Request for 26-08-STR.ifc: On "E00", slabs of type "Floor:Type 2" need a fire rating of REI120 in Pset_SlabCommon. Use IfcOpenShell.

First a look at what the model holds.

```python
import ifcopenshell
import ifcopenshell.util.element

model = ifcopenshell.open("26-08-STR.ifc")
print(model.schema)
storey = next(s for s in model.by_type("IfcBuildingStorey") if s.Name == "E00")
slabs = [e for e in ifcopenshell.util.element.get_decomposition(storey) if e.is_a("IfcSlab")]
seen = {}
for e in slabs:
    element_type = ifcopenshell.util.element.get_type(e)
    key = (element_type.Name if element_type != e and element_type else None, ifcopenshell.util.element.get_pset(e, "Pset_SlabCommon", "FireRating"))
    seen[key] = seen.get(key, 0) + 1
for (name, value), count in sorted(seen.items(), key=str):
    print(count, "x", name, "|", value)
```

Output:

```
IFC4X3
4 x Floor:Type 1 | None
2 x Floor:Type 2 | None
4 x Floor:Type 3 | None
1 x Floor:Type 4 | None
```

```python
import ifcopenshell
import ifcopenshell.api.pset
import ifcopenshell.util.element

model = ifcopenshell.open("26-08-STR.ifc")

storey = next(s for s in model.by_type("IfcBuildingStorey") if s.Name == "E00")
slabs = [e for e in ifcopenshell.util.element.get_decomposition(storey) if e.is_a("IfcSlab")]

count = 0
for e in slabs:
    element_type = ifcopenshell.util.element.get_type(e)
    if element_type in (None, e) or element_type.Name != "Floor:Type 2":
        continue
    # add_pset returns the element's existing set when there is one.
    pset = ifcopenshell.api.pset.add_pset(model, product=e, name="Pset_SlabCommon")
    ifcopenshell.api.pset.edit_pset(model, pset=pset, properties={"FireRating": "REI120"})
    count += 1

print(count, "slabs updated")

model.write("26-08-STR_rev.ifc")
```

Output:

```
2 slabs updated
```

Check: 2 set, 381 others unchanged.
